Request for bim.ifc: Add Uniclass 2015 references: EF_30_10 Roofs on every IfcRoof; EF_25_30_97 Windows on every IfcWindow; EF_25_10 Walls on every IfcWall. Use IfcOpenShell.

First a look at what the model holds.

```python
import ifcopenshell

model = ifcopenshell.open("bim.ifc")
print(model.schema)
print("classifications:", [c.Name for c in model.by_type("IfcClassification")])
for ifc_class in ("IfcDoor", "IfcRoof", "IfcStair", "IfcWall", "IfcWindow"):
    print(ifc_class, len(model.by_type(ifc_class)))
```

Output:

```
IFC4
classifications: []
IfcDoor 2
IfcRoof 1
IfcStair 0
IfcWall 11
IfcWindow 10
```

```python
import ifcopenshell
import ifcopenshell.api.classification

model = ifcopenshell.open("bim.ifc")

system = ifcopenshell.api.classification.add_classification(model, classification="Uniclass 2015")

codes = {
    "IfcRoof": ("EF_30_10", "Roofs"),
    "IfcWindow": ("EF_25_30_97", "Windows"),
    "IfcWall": ("EF_25_10", "Walls"),
}
for ifc_class, (code, name) in codes.items():
    products = model.by_type(ifc_class)
    ifcopenshell.api.classification.add_reference(
        model, products=products, classification=system, identification=code, name=name
    )
    print(code, len(products))

model.write("bim_rev.ifc")
```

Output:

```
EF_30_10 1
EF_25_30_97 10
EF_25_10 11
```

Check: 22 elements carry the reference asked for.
